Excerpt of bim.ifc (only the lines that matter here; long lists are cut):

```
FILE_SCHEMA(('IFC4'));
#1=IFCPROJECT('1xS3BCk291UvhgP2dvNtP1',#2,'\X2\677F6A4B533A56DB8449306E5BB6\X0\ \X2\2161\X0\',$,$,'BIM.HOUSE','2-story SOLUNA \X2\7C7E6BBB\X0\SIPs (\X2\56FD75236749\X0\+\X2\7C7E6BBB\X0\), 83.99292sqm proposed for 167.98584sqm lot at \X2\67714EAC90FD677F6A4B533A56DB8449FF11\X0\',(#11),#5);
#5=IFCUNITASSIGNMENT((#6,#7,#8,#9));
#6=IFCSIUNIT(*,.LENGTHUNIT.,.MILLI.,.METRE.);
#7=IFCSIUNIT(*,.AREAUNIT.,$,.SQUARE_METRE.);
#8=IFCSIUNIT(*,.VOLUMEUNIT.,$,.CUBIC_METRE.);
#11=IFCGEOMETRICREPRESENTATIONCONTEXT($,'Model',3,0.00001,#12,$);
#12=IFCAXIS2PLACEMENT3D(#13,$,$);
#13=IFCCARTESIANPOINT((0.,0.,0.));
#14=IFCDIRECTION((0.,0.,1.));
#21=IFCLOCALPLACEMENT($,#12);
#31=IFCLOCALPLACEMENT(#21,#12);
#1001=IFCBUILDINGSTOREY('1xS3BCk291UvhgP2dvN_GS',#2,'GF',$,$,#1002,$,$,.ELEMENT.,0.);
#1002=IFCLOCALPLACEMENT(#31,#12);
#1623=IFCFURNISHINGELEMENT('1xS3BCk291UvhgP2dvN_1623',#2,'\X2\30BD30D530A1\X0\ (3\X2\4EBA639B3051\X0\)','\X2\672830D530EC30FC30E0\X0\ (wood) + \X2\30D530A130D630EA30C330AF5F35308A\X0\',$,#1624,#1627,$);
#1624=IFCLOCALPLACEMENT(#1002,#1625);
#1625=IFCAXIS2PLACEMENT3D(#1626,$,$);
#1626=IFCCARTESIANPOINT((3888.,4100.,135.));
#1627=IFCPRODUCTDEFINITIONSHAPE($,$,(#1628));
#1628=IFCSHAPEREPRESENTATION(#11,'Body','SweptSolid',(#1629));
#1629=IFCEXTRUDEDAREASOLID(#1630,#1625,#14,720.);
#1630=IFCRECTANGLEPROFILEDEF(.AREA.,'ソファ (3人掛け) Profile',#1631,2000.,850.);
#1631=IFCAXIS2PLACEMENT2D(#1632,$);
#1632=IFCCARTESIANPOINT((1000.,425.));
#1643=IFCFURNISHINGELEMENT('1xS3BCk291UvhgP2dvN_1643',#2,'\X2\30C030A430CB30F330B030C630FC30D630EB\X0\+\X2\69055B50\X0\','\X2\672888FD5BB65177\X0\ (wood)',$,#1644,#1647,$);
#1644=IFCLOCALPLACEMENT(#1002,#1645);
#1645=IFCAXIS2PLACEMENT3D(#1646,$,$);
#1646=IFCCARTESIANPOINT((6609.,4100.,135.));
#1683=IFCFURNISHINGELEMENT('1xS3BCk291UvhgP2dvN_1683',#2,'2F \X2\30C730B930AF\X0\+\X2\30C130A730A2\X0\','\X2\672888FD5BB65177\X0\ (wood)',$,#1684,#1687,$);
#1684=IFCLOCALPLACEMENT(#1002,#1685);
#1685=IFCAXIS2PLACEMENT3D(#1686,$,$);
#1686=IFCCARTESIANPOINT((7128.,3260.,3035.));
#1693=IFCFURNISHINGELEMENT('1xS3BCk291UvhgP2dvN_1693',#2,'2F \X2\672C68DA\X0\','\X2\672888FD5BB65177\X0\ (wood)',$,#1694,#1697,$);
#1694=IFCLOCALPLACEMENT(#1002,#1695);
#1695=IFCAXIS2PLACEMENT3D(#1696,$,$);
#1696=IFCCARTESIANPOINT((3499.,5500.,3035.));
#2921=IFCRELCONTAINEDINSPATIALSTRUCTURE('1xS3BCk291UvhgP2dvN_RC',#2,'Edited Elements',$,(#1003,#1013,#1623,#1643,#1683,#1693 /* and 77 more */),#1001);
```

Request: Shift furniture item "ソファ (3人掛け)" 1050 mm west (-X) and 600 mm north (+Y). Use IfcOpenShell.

```python
import ifcopenshell
import ifcopenshell.api.geometry
import ifcopenshell.util.placement

model = ifcopenshell.open("bim.ifc")

item = model.by_guid("1xS3BCk291UvhgP2dvN_1623")
matrix = ifcopenshell.util.placement.get_local_placement(item.ObjectPlacement)
matrix[0, 3] -= 1050.0
matrix[1, 3] += 600.0
ifcopenshell.api.geometry.edit_object_placement(model, product=item, matrix=matrix, is_si=False)

print(ifcopenshell.util.placement.get_local_placement(item.ObjectPlacement).round(3) + 0.0)

model.write("bim_updated.ifc")
```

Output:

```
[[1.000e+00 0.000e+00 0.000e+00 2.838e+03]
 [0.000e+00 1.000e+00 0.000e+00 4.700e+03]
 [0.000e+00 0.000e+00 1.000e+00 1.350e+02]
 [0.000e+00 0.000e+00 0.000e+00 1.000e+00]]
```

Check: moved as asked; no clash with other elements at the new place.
